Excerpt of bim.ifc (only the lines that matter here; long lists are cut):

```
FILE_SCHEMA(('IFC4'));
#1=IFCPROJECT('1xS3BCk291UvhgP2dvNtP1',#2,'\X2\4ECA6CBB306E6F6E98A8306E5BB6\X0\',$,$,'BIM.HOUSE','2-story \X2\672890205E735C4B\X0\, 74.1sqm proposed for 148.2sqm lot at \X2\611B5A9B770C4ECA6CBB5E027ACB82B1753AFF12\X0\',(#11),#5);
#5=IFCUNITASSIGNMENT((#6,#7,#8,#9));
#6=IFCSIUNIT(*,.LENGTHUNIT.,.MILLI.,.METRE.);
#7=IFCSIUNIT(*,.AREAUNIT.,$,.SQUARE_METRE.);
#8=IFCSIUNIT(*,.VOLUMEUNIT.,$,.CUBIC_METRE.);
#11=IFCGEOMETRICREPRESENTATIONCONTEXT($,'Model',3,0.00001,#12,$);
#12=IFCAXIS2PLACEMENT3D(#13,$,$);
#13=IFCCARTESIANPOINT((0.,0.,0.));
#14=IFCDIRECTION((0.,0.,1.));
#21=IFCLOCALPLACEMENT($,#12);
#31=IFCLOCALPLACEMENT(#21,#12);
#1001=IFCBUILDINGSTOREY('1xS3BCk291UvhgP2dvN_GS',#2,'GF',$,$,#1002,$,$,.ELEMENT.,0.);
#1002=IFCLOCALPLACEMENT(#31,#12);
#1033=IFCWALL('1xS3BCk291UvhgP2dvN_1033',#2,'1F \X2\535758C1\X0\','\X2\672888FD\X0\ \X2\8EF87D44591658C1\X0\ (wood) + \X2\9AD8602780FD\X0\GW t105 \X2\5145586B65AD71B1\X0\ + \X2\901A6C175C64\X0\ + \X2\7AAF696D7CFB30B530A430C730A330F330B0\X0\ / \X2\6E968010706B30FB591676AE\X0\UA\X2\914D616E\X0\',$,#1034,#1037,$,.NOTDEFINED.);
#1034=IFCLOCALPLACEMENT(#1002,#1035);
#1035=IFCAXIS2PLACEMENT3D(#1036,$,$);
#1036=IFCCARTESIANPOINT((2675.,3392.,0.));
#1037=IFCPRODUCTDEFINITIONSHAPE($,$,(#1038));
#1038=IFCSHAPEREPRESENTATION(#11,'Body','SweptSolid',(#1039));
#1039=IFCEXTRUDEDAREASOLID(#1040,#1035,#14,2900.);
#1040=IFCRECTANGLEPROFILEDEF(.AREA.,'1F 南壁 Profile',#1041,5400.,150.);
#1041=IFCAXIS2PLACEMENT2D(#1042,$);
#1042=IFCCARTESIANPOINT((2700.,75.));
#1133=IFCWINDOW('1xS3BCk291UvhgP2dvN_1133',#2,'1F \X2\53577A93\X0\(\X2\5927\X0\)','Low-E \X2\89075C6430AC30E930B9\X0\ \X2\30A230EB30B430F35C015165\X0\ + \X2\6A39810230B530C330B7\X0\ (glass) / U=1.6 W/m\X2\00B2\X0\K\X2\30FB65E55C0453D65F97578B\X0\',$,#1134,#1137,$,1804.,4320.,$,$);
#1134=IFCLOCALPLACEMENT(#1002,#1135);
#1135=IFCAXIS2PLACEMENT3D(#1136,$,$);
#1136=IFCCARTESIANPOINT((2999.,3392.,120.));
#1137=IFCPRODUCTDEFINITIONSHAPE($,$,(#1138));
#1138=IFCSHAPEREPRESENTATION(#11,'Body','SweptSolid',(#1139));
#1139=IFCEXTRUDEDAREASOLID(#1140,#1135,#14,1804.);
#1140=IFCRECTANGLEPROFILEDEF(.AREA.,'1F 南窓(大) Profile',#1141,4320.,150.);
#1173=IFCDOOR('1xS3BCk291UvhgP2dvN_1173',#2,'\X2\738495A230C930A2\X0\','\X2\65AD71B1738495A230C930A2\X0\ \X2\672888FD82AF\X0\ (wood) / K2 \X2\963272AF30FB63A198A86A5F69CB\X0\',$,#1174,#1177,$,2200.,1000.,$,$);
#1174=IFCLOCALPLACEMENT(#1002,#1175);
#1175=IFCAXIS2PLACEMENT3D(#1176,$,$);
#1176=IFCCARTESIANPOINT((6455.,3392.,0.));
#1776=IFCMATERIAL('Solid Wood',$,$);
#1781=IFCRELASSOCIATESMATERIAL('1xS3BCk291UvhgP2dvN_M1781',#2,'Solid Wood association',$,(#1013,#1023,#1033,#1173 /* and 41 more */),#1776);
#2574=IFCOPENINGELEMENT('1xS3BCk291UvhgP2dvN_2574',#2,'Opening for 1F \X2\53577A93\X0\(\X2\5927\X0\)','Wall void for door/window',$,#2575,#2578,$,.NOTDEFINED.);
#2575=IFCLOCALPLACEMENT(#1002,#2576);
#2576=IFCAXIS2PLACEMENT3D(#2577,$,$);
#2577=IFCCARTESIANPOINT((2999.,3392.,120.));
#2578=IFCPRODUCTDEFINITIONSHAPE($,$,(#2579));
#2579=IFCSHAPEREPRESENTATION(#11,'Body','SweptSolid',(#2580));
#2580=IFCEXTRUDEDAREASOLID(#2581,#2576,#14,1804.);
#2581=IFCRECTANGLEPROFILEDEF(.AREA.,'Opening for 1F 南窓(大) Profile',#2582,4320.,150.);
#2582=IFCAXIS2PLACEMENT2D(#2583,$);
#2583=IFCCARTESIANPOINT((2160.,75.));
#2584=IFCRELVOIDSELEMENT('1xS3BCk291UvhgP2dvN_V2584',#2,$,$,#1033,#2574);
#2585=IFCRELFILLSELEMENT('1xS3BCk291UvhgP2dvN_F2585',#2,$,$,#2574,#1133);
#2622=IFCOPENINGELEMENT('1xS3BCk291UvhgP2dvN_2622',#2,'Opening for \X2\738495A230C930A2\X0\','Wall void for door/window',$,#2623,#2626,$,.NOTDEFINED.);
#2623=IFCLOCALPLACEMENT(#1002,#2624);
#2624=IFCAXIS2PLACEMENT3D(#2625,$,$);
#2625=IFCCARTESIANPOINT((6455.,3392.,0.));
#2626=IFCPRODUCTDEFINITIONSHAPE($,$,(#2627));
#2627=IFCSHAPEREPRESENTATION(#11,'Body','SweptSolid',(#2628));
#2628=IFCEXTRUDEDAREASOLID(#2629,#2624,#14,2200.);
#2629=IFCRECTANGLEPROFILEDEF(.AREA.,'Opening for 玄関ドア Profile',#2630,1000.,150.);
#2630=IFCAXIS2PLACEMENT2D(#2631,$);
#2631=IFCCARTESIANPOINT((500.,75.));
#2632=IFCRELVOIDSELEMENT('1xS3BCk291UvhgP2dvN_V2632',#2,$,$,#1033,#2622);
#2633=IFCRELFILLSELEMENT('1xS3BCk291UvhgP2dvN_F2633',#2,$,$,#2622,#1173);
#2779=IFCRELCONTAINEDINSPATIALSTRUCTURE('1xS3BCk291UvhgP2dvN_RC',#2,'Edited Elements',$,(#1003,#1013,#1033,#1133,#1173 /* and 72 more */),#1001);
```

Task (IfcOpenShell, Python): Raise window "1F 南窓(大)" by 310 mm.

```python
import numpy as np
import ifcopenshell
import ifcopenshell.api.geometry
import ifcopenshell.util.placement
import ifcopenshell.util.unit

model = ifcopenshell.open("bim.ifc")
unit_scale = ifcopenshell.util.unit.calculate_unit_scale(model)

window = model.by_guid("1xS3BCk291UvhgP2dvN_1133")
opening = window.FillsVoids[0].RelatingOpeningElement
dz = 310.0

shift = np.array([0.0, 0.0, dz])
# The window is not placed relative to its opening, so move both.
for product in (opening, window):
    matrix = ifcopenshell.util.placement.get_local_placement(product.ObjectPlacement)
    matrix[:3, 3] += shift
    ifcopenshell.api.geometry.edit_object_placement(model, product=product, matrix=matrix, is_si=False)

print(f"moved by {dz * unit_scale:+.3f} m")

model.write("bim_rev.ifc")
```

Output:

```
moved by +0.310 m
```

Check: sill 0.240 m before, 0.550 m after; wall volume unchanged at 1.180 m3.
